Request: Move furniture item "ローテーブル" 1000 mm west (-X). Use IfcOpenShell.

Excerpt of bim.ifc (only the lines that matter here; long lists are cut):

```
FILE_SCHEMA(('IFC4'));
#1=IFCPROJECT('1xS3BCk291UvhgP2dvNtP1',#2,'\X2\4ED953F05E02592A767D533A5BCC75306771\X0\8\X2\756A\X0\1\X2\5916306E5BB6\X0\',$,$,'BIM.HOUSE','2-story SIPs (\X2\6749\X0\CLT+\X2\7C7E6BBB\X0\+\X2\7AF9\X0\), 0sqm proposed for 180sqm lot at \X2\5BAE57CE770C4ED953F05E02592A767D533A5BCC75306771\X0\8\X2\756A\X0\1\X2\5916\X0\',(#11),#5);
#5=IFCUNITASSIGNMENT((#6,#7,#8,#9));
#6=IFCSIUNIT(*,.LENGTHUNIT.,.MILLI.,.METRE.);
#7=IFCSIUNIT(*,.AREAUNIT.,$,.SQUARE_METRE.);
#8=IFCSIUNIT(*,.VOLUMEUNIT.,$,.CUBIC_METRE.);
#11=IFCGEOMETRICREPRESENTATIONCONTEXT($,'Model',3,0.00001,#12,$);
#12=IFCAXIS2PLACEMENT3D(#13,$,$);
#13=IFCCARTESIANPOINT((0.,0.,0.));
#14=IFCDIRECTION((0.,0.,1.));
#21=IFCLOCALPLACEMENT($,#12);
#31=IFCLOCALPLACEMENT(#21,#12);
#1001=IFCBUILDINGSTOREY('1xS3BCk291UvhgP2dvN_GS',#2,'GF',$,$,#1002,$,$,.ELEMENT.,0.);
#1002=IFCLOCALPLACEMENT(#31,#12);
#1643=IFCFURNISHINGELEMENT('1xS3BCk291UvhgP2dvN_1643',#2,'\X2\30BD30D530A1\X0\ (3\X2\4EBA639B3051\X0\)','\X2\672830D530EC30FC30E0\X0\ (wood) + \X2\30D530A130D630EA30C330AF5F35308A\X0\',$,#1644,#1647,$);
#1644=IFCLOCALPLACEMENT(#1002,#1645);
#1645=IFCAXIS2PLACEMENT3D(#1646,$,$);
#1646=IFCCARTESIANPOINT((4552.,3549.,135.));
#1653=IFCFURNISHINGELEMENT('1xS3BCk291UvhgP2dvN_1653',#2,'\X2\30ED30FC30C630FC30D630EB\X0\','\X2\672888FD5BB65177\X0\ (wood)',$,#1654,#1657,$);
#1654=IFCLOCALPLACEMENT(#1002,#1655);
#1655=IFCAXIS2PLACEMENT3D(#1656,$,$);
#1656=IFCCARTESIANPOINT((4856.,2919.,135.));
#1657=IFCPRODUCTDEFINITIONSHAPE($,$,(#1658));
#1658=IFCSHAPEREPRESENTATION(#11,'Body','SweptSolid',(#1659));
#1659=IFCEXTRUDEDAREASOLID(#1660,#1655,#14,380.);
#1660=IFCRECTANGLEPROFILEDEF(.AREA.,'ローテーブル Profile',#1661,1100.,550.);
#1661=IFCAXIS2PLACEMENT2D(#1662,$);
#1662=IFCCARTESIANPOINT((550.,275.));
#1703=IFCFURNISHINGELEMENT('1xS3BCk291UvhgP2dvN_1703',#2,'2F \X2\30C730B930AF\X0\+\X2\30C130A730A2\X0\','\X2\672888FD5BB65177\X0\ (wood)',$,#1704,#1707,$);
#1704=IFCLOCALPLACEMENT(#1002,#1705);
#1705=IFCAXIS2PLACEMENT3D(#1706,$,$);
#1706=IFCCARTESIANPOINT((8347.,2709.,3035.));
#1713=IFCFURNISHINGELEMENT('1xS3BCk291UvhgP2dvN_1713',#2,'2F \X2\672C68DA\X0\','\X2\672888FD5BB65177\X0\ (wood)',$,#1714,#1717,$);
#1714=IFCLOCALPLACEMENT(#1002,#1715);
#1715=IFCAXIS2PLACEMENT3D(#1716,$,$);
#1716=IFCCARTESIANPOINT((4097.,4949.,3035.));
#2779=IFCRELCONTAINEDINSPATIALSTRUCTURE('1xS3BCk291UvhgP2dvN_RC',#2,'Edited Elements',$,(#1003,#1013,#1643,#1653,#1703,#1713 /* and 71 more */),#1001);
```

```python
import ifcopenshell
import ifcopenshell.api.geometry
import ifcopenshell.util.placement

model = ifcopenshell.open("bim.ifc")

item = model.by_guid("1xS3BCk291UvhgP2dvN_1653")
matrix = ifcopenshell.util.placement.get_local_placement(item.ObjectPlacement)
matrix[0, 3] -= 1000.0
ifcopenshell.api.geometry.edit_object_placement(model, product=item, matrix=matrix, is_si=False)

print(ifcopenshell.util.placement.get_local_placement(item.ObjectPlacement).round(3) + 0.0)

model.write("bim-out.ifc")
```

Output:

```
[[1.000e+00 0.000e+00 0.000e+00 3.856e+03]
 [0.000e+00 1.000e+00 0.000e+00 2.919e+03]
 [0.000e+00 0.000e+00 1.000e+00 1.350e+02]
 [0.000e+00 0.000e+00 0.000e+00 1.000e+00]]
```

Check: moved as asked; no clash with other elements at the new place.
